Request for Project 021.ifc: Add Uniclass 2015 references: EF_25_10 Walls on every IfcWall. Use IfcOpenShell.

First a look at what the model holds.

```python
import ifcopenshell

model = ifcopenshell.open("Project 021.ifc")
print(model.schema)
print("classifications:", [c.Name for c in model.by_type("IfcClassification")])
for ifc_class in ("IfcDoor", "IfcRoof", "IfcStair", "IfcWall", "IfcWindow"):
    print(ifc_class, len(model.by_type(ifc_class)))
```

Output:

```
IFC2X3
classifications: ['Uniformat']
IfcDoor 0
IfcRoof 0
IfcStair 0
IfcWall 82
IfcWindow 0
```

```python
import ifcopenshell
import ifcopenshell.api.classification

model = ifcopenshell.open("Project 021.ifc")

# IFC2X3 requires Source and Edition and has no link from the project to the system.
system = model.create_entity("IfcClassification", Source="NBS", Edition="2015", Name="Uniclass 2015")

codes = {
    "IfcWall": ("EF_25_10", "Walls"),
}
for ifc_class, (code, name) in codes.items():
    products = model.by_type(ifc_class)
    ifcopenshell.api.classification.add_reference(
        model, products=products, classification=system, identification=code, name=name
    )
    print(code, len(products))

model.write("Project 021_v2.ifc")
```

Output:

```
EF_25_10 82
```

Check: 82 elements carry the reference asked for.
